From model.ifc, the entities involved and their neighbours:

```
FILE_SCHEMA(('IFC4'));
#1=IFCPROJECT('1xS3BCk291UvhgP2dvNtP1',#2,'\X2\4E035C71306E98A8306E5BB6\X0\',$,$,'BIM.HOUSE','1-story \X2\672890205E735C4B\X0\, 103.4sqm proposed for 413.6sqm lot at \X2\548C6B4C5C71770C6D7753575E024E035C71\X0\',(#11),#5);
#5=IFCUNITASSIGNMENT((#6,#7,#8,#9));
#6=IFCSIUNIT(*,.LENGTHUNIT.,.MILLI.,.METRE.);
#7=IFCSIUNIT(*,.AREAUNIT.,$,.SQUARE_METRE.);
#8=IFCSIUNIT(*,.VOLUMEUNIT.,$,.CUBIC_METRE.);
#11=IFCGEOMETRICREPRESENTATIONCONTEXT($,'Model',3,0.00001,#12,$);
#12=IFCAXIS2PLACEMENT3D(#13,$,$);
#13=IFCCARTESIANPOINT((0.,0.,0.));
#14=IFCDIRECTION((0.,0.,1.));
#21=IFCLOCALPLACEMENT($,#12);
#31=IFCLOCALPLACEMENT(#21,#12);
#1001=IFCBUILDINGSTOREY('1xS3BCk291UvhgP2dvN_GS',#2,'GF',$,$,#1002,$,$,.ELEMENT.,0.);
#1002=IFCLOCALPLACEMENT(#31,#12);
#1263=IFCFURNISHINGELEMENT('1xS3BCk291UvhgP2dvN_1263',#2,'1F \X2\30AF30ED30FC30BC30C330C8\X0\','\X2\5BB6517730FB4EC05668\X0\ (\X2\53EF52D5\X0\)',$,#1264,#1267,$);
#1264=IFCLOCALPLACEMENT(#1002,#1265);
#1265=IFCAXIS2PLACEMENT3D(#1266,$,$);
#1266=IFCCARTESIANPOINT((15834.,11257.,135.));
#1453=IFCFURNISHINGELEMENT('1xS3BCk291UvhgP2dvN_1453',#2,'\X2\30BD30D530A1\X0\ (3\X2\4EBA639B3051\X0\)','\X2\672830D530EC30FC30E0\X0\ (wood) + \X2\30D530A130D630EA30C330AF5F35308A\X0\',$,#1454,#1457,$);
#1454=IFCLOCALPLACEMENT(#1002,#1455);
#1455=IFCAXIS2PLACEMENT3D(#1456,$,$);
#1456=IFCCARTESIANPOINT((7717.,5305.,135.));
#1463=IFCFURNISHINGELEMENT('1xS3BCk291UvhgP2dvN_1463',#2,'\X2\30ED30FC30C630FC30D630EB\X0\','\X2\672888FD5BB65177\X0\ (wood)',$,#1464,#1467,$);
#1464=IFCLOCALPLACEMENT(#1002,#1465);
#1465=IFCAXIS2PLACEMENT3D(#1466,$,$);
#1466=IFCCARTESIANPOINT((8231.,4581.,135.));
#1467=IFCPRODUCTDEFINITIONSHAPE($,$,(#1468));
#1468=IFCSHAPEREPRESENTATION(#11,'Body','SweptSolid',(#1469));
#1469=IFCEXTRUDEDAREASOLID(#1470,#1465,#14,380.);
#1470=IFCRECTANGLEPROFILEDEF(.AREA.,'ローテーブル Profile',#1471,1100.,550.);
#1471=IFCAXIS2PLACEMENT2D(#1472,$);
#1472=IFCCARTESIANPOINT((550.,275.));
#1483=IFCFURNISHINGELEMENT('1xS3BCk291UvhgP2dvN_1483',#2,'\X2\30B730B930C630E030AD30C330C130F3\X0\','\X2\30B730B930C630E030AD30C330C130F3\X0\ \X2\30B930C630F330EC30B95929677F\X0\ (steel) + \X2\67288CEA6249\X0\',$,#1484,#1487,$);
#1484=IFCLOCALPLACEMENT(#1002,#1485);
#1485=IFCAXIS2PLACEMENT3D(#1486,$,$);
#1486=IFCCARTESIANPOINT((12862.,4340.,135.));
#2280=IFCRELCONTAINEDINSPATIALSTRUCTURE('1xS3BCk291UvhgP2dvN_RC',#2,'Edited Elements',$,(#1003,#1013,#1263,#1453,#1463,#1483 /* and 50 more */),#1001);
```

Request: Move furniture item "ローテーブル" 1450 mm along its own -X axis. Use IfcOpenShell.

```python
import ifcopenshell
import ifcopenshell.api.geometry
import ifcopenshell.util.placement

model = ifcopenshell.open("model.ifc")

item = model.by_guid("1xS3BCk291UvhgP2dvN_1463")
matrix = ifcopenshell.util.placement.get_local_placement(item.ObjectPlacement)
matrix[:3, 3] -= matrix[:3, 0] * 1450.0
ifcopenshell.api.geometry.edit_object_placement(model, product=item, matrix=matrix, is_si=False)

print(ifcopenshell.util.placement.get_local_placement(item.ObjectPlacement).round(3) + 0.0)

model.write("model_v2.ifc")
```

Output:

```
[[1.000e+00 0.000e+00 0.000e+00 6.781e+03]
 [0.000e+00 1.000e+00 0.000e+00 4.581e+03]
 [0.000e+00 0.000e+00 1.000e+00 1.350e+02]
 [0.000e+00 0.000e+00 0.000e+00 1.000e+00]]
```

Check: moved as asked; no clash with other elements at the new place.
